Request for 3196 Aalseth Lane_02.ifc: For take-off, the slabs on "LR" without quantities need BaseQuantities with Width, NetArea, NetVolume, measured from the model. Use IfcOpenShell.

First a look at what the model holds.

```python
import ifcopenshell
import ifcopenshell.util.element
import ifcopenshell.util.unit

model = ifcopenshell.open("3196 Aalseth Lane_02.ifc")
print(model.schema)
for unit_type in ("LENGTHUNIT", "AREAUNIT", "VOLUMEUNIT"):
    print(unit_type, ifcopenshell.util.unit.calculate_unit_scale(model, unit_type))
storey = next(s for s in model.by_type("IfcBuildingStorey") if s.Name == "LR")
slabs = [e for e in ifcopenshell.util.element.get_decomposition(storey) if e.is_a("IfcSlab")]
for e in sorted(slabs, key=lambda e: e.id()):
    print(e.id(), e.is_a(), e.Name, list(ifcopenshell.util.element.get_psets(e, qtos_only=True)), sep=" | ")
```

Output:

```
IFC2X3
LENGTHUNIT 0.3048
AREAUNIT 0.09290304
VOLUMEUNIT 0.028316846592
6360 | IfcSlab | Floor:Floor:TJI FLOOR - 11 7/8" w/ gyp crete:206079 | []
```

```python
import ifcopenshell
import ifcopenshell.api.pset
import ifcopenshell.geom
import ifcopenshell.util.element
import ifcopenshell.util.shape
import ifcopenshell.util.unit

model = ifcopenshell.open("3196 Aalseth Lane_02.ifc")
unit_scale = ifcopenshell.util.unit.calculate_unit_scale(model)
area_scale = ifcopenshell.util.unit.calculate_unit_scale(model, "AREAUNIT")
volume_scale = ifcopenshell.util.unit.calculate_unit_scale(model, "VOLUMEUNIT")
settings = ifcopenshell.geom.settings()

storey = next(s for s in model.by_type("IfcBuildingStorey") if s.Name == "LR")
slabs = [e for e in ifcopenshell.util.element.get_decomposition(storey) if e.is_a("IfcSlab")]

for e in sorted(slabs, key=lambda e: e.id()):
    if ifcopenshell.util.element.get_psets(e, qtos_only=True, should_inherit=False):
        continue
    # Geometry comes back in metres, in the element's own axes.
    shape = ifcopenshell.geom.create_shape(settings, e)
    values = {
        "Width": ifcopenshell.util.shape.get_z(shape.geometry) / unit_scale,
        "NetArea": ifcopenshell.util.shape.get_footprint_area(shape.geometry) / area_scale,
        "NetVolume": ifcopenshell.util.shape.get_volume(shape.geometry) / volume_scale,
    }
    qto = ifcopenshell.api.pset.add_qto(model, product=e, name="BaseQuantities")
    ifcopenshell.api.pset.edit_qto(model, qto=qto, properties=values)
    print(e.id(), {k: round(v, 3) for k, v in values.items()})

model.write("3196 Aalseth Lane_02_rev.ifc")
```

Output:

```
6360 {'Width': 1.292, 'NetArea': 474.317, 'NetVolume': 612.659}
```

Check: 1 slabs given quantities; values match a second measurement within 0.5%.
